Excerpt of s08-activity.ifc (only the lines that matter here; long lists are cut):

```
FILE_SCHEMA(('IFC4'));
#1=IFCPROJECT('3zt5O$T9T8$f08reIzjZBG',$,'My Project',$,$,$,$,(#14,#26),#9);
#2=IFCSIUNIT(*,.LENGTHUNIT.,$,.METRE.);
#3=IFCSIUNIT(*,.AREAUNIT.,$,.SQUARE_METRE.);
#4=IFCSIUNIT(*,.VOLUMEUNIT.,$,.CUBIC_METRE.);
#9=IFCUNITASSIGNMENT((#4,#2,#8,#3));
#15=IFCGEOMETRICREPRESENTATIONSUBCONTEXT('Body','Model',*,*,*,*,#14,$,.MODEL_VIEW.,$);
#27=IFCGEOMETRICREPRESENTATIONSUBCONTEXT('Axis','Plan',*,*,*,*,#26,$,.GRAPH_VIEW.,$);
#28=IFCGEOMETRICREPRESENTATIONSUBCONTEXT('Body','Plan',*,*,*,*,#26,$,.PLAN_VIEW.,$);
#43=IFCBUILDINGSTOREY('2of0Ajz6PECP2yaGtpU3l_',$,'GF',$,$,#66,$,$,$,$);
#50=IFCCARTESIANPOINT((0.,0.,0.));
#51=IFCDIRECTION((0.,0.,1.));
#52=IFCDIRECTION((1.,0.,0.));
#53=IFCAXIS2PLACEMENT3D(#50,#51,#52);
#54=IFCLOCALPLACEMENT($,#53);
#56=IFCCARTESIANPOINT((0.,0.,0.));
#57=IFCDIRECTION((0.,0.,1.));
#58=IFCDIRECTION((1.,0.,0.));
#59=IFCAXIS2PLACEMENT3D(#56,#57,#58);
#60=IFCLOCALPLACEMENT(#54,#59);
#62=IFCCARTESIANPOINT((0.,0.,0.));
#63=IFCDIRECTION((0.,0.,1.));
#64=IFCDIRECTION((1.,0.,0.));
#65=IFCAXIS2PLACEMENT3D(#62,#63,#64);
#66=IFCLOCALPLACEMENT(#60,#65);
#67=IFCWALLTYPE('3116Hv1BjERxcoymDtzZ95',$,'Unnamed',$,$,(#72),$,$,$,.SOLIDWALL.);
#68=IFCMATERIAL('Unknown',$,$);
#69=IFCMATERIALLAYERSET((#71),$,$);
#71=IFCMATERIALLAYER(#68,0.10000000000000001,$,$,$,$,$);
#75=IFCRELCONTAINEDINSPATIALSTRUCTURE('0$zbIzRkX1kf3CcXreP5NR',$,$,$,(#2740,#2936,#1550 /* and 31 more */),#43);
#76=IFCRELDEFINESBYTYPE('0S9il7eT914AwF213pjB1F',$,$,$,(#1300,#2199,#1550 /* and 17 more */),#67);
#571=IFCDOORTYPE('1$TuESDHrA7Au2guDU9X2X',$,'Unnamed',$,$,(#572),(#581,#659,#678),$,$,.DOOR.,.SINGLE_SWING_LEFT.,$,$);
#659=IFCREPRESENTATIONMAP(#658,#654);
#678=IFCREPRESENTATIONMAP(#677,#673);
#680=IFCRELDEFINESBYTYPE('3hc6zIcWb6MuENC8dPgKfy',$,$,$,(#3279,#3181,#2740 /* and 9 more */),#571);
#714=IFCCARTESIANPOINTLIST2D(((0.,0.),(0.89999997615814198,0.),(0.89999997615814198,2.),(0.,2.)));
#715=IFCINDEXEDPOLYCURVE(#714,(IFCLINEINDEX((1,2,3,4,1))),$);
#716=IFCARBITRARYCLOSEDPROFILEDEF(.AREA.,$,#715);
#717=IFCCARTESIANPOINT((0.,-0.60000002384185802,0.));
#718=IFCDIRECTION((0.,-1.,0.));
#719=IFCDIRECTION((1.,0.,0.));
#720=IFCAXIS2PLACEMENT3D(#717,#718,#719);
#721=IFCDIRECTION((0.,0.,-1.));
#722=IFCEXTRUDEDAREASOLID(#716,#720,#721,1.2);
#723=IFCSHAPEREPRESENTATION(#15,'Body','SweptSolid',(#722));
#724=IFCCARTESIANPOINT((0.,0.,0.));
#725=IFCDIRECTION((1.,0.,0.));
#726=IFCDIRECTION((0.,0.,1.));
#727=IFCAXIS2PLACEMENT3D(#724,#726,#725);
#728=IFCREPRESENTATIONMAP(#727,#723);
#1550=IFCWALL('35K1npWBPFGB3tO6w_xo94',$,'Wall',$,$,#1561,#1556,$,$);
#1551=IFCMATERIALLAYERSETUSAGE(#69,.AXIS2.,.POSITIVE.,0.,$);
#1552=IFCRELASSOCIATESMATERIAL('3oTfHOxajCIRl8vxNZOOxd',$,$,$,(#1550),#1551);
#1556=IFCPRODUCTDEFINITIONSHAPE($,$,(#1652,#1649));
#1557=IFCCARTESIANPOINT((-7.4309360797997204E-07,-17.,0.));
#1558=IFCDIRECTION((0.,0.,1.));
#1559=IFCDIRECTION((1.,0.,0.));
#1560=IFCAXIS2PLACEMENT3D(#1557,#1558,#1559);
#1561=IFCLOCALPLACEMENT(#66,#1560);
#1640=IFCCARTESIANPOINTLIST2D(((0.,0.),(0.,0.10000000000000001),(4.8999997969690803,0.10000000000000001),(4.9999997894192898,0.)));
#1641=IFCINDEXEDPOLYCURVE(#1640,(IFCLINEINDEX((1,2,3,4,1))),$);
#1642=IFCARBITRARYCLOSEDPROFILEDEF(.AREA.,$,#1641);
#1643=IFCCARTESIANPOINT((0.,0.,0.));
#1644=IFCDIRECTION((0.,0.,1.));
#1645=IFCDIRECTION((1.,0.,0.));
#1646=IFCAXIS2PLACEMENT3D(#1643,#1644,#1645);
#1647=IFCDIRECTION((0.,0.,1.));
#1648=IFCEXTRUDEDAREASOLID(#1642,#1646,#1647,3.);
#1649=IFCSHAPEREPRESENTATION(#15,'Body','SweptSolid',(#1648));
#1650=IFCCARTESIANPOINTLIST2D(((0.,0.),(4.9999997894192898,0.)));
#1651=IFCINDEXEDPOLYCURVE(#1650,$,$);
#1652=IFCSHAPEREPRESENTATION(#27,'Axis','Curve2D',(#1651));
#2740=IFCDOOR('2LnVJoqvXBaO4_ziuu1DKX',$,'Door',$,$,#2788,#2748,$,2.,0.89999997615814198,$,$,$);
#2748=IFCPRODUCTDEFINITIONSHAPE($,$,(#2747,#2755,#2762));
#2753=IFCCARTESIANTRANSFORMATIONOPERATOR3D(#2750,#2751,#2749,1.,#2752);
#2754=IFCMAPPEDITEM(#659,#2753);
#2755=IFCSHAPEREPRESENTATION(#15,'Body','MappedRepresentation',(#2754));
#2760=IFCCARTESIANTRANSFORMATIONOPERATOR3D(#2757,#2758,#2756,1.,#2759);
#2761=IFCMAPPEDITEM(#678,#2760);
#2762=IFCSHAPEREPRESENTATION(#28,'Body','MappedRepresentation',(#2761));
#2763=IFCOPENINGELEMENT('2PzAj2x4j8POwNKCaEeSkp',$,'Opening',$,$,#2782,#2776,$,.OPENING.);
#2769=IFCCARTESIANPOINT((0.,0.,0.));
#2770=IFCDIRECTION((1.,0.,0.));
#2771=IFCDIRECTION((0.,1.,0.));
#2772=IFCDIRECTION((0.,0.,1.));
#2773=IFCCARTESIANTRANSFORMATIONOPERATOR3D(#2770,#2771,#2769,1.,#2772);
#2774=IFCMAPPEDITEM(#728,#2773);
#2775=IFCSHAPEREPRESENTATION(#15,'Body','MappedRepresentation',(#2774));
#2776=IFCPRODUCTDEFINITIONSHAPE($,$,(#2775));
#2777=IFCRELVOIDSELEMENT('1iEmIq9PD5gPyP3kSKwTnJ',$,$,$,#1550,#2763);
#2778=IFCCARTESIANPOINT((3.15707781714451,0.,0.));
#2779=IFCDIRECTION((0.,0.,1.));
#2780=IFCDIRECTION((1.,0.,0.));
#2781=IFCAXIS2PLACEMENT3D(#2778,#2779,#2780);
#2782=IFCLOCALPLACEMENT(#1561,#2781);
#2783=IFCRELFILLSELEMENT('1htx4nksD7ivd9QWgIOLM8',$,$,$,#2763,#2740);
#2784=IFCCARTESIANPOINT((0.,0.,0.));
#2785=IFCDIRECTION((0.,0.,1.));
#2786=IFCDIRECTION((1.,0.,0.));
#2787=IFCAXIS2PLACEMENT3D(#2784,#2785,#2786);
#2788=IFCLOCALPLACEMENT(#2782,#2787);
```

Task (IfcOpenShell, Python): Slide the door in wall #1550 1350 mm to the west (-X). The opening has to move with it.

```python
import ifcopenshell
import ifcopenshell.api.geometry
import ifcopenshell.util.placement

model = ifcopenshell.open("s08-activity.ifc")

door = model.by_guid("2LnVJoqvXBaO4_ziuu1DKX")
opening = door.FillsVoids[0].RelatingOpeningElement
wall = opening.VoidsElements[0].RelatingBuildingElement

wall_matrix = ifcopenshell.util.placement.get_local_placement(wall.ObjectPlacement)
shift = wall_matrix[:3, 0] * -1.35
before = ifcopenshell.util.placement.get_local_placement(door.ObjectPlacement)[:3, 3].copy()

# The door is placed relative to its opening, so it follows when the opening moves.
matrix = ifcopenshell.util.placement.get_local_placement(opening.ObjectPlacement)
matrix[:3, 3] += shift
ifcopenshell.api.geometry.edit_object_placement(
    model, product=opening, matrix=matrix, is_si=False, should_transform_children=True
)

after = ifcopenshell.util.placement.get_local_placement(door.ObjectPlacement)[:3, 3]
print("door moved by", (after - before).round(3) + 0.0)

model.write("s08-activity_updated.ifc")
```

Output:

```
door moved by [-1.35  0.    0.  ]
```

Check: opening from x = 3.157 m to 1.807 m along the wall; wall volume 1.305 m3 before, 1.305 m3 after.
